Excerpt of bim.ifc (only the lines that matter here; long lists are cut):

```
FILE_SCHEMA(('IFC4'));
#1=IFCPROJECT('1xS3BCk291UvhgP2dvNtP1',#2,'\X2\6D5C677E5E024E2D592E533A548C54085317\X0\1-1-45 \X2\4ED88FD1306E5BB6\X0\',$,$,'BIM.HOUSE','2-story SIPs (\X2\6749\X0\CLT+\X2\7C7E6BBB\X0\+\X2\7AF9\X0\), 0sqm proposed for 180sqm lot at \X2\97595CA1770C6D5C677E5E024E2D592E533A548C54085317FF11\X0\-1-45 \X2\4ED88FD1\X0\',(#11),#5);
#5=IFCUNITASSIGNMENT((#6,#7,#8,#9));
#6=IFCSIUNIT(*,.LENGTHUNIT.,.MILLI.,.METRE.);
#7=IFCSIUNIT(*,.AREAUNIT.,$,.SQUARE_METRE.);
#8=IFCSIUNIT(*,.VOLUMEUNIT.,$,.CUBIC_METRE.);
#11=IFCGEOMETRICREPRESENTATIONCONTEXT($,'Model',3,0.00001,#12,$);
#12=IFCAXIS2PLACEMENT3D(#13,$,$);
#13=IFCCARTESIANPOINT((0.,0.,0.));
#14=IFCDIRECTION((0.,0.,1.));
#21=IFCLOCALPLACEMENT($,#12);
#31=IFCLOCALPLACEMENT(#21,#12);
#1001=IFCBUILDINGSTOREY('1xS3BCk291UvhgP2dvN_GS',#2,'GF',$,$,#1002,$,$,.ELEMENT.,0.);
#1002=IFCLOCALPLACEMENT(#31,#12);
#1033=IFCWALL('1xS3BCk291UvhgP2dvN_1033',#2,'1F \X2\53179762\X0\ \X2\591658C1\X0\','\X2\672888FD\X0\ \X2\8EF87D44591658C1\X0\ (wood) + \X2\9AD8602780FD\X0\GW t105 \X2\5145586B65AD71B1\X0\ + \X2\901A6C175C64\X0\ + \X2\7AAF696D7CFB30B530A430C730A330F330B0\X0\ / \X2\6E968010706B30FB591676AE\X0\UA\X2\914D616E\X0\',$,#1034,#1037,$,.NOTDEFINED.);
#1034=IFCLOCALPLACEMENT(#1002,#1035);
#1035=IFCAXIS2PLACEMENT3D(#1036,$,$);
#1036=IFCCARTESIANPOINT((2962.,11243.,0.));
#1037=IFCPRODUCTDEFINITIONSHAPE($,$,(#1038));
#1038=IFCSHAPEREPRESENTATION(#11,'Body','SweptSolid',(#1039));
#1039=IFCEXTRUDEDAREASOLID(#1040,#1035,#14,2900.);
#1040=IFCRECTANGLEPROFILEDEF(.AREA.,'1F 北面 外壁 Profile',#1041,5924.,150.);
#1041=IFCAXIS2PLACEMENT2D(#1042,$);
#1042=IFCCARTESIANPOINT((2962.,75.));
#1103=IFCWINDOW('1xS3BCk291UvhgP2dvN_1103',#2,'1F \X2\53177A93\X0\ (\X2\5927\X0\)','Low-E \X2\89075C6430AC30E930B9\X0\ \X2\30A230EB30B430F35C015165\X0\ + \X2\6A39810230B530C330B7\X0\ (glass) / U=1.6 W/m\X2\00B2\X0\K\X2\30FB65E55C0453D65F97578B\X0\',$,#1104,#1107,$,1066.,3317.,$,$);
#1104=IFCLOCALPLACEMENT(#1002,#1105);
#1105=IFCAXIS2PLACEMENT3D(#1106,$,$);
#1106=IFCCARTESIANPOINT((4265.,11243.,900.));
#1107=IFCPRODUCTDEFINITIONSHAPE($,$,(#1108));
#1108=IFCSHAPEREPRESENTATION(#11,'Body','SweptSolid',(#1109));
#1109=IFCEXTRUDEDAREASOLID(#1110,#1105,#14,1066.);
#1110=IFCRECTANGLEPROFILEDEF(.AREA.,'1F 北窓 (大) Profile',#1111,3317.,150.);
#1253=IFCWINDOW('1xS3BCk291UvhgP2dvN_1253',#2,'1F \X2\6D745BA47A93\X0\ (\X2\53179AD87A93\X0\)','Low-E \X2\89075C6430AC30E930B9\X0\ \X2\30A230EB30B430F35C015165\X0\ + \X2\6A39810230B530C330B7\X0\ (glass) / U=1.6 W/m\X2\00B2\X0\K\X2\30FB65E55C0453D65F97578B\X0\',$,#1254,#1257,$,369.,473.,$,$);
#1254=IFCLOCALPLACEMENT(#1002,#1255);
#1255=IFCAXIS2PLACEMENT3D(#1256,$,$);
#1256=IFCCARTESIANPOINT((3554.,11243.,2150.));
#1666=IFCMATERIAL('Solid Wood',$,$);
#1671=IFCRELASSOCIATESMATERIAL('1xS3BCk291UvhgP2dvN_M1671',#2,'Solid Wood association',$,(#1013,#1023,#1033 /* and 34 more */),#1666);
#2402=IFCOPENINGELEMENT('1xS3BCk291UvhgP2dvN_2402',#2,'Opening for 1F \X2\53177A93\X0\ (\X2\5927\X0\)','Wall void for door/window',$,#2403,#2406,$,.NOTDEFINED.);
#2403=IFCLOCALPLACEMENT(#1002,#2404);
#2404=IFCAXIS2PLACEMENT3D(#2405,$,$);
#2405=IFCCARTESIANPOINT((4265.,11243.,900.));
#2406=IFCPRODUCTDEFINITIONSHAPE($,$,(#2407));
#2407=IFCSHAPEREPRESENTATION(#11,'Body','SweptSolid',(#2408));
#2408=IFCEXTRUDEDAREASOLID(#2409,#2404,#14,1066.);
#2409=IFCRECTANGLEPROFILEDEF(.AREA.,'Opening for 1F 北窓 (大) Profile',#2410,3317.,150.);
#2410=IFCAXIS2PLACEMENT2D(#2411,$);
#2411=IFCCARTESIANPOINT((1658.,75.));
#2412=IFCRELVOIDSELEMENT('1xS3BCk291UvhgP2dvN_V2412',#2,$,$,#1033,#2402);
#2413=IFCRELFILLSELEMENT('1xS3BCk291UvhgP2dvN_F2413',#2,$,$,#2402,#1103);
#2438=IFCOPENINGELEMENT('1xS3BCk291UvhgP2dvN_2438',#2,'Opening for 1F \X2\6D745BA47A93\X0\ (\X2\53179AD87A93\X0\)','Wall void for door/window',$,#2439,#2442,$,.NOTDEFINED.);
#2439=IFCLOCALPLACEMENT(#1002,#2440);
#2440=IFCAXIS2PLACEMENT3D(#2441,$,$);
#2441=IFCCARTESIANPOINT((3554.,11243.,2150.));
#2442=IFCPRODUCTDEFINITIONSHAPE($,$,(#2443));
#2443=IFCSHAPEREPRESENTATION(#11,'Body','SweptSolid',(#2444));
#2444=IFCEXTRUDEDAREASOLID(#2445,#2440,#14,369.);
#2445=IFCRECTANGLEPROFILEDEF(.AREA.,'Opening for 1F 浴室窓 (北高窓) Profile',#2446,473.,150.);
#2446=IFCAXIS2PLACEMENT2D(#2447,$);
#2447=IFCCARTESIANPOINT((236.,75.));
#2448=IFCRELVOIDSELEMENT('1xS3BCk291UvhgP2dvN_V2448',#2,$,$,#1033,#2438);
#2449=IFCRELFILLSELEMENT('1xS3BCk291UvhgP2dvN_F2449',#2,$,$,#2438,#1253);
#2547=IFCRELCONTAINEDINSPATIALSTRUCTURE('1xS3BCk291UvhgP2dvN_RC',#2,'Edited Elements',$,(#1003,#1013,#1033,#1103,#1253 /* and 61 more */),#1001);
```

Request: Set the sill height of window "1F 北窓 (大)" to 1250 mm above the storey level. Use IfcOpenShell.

```python
import numpy as np
import ifcopenshell
import ifcopenshell.api.geometry
import ifcopenshell.geom
import ifcopenshell.util.element
import ifcopenshell.util.placement
import ifcopenshell.util.shape
import ifcopenshell.util.unit

model = ifcopenshell.open("bim.ifc")
unit_scale = ifcopenshell.util.unit.calculate_unit_scale(model)

window = model.by_id(1103)
opening = window.FillsVoids[0].RelatingOpeningElement
storey = ifcopenshell.util.element.get_container(window, ifc_class="IfcBuildingStorey")
level = ifcopenshell.util.placement.get_local_placement(storey.ObjectPlacement)[2, 3]

# The opening's origin need not be at the sill, so measure its lowest point.
shape = ifcopenshell.geom.create_shape(ifcopenshell.geom.settings(), opening)
bottom = ifcopenshell.util.shape.get_shape_bottom_elevation(shape, shape.geometry) / unit_scale
dz = level + 1.25 / unit_scale - bottom

shift = np.array([0.0, 0.0, dz])
# The window is not placed relative to its opening, so move both.
for product in (opening, window):
    matrix = ifcopenshell.util.placement.get_local_placement(product.ObjectPlacement)
    matrix[:3, 3] += shift
    ifcopenshell.api.geometry.edit_object_placement(model, product=product, matrix=matrix, is_si=False)

print(f"moved by {dz * unit_scale:+.3f} m")

model.write("bim-out.ifc")
```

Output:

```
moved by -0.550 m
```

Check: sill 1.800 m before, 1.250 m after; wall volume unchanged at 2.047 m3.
